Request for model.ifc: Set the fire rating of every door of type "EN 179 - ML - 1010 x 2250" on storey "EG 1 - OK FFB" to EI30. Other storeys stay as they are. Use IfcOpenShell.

First a look at what the model holds.

```python
import ifcopenshell
import ifcopenshell.util.element

model = ifcopenshell.open("model.ifc")
print(model.schema)
storey = next(s for s in model.by_type("IfcBuildingStorey") if s.Name == "EG 1 - OK FFB")
doors = [e for e in ifcopenshell.util.element.get_decomposition(storey) if e.is_a("IfcDoor")]
seen = {}
for e in doors:
    element_type = ifcopenshell.util.element.get_type(e)
    key = (element_type.Name if element_type != e and element_type else None, ifcopenshell.util.element.get_pset(e, "Pset_DoorCommon", "FireRating"))
    seen[key] = seen.get(key, 0) + 1
for (name, value), count in sorted(seen.items(), key=str):
    print(count, "x", name, "|", value)
```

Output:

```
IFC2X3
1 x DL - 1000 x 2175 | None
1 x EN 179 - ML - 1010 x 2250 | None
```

```python
import ifcopenshell
import ifcopenshell.api.pset
import ifcopenshell.util.element

model = ifcopenshell.open("model.ifc")

storey = next(s for s in model.by_type("IfcBuildingStorey") if s.Name == "EG 1 - OK FFB")
doors = [e for e in ifcopenshell.util.element.get_decomposition(storey) if e.is_a("IfcDoor")]

count = 0
for e in doors:
    element_type = ifcopenshell.util.element.get_type(e)
    if element_type in (None, e) or element_type.Name != "EN 179 - ML - 1010 x 2250":
        continue
    # add_pset returns the element's existing set when there is one.
    pset = ifcopenshell.api.pset.add_pset(model, product=e, name="Pset_DoorCommon")
    ifcopenshell.api.pset.edit_pset(model, pset=pset, properties={"FireRating": "EI30"})
    count += 1

print(count, "doors updated")

model.write("model_rev.ifc")
```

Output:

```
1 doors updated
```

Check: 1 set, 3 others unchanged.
